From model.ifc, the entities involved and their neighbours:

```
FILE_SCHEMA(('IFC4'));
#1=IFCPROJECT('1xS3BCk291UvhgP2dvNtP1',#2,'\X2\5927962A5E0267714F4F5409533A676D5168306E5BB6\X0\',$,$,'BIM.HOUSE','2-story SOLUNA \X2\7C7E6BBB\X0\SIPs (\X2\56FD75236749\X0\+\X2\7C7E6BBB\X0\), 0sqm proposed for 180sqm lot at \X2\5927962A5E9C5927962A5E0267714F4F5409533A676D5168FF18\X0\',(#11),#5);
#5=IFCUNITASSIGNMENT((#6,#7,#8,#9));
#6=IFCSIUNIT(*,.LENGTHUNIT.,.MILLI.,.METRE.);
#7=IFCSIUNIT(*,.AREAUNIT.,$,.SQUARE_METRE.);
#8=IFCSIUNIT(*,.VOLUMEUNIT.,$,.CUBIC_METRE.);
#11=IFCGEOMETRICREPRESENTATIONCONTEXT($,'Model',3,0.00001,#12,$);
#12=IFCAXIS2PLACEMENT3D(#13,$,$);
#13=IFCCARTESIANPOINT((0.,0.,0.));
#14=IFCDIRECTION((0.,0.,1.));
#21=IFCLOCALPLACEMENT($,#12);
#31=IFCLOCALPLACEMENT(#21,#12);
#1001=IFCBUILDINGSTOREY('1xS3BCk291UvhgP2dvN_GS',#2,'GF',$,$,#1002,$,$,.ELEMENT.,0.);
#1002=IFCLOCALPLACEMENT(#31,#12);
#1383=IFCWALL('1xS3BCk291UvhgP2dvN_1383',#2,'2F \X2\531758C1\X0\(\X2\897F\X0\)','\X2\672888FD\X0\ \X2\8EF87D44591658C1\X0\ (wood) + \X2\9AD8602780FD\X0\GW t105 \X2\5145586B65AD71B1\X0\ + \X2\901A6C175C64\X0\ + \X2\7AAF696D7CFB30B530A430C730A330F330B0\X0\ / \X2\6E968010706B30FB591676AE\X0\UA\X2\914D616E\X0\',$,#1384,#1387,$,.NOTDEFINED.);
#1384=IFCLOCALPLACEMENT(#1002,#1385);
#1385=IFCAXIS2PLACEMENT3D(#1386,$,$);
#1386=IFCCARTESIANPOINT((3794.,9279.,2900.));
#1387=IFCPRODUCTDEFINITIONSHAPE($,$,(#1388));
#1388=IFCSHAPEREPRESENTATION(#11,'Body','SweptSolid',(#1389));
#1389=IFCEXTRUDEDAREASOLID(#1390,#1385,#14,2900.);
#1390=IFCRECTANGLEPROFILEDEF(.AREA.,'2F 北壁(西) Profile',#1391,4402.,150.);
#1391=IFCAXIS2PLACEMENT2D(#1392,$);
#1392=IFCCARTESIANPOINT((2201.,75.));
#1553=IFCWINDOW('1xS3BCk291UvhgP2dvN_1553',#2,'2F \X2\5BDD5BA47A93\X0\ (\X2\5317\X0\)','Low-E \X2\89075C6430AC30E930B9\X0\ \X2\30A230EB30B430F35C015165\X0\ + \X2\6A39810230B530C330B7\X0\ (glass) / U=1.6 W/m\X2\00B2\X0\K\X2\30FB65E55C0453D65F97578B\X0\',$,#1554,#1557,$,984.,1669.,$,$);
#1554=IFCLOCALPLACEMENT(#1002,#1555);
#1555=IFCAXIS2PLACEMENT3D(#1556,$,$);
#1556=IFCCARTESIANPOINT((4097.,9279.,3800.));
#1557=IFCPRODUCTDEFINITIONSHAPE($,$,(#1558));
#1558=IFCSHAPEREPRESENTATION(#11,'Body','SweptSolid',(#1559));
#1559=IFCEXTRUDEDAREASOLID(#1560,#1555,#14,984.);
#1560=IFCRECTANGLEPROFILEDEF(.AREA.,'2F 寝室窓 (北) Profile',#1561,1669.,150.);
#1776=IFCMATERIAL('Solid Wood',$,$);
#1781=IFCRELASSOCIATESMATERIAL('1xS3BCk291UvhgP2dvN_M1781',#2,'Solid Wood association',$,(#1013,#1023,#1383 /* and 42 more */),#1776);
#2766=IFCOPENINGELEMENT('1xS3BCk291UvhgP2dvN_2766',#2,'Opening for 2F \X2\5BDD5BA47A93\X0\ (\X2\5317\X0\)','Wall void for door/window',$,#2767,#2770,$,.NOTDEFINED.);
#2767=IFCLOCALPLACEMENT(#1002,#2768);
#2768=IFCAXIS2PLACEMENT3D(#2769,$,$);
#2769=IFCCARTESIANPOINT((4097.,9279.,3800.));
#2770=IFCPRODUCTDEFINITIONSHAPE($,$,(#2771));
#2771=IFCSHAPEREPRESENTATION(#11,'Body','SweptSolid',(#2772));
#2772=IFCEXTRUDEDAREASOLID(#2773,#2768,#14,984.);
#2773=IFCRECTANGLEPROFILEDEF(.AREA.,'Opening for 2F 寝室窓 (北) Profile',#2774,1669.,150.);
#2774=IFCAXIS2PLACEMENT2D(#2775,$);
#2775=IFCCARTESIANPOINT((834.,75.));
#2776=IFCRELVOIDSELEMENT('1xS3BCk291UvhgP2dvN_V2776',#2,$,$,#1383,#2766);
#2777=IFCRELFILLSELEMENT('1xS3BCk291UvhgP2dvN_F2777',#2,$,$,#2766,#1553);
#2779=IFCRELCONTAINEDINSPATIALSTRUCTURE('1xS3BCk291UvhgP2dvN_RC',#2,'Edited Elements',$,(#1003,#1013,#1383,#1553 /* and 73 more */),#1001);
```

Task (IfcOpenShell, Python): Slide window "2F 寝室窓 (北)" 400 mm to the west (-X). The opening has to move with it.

```python
import ifcopenshell
import ifcopenshell.api.geometry
import ifcopenshell.util.placement

model = ifcopenshell.open("model.ifc")

window = model.by_guid("1xS3BCk291UvhgP2dvN_1553")
opening = window.FillsVoids[0].RelatingOpeningElement
wall = opening.VoidsElements[0].RelatingBuildingElement

wall_matrix = ifcopenshell.util.placement.get_local_placement(wall.ObjectPlacement)
shift = wall_matrix[:3, 0] * -400.0
before = ifcopenshell.util.placement.get_local_placement(window.ObjectPlacement)[:3, 3].copy()

# The window is not placed relative to its opening, so move both.
for product in (opening, window):
    matrix = ifcopenshell.util.placement.get_local_placement(product.ObjectPlacement)
    matrix[:3, 3] += shift
    ifcopenshell.api.geometry.edit_object_placement(model, product=product, matrix=matrix, is_si=False)

after = ifcopenshell.util.placement.get_local_placement(window.ObjectPlacement)[:3, 3]
print("window moved by", (after - before).round(3) + 0.0)

model.write("model-out.ifc")
```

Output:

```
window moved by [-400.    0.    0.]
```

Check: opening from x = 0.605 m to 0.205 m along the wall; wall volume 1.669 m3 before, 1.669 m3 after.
